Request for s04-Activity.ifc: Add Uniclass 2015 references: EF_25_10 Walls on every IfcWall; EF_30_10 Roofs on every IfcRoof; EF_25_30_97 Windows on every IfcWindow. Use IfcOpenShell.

First a look at what the model holds.

```python
import ifcopenshell

model = ifcopenshell.open("s04-Activity.ifc")
print(model.schema)
print("classifications:", [c.Name for c in model.by_type("IfcClassification")])
for ifc_class in ("IfcDoor", "IfcRoof", "IfcStair", "IfcWall", "IfcWindow"):
    print(ifc_class, len(model.by_type(ifc_class)))
```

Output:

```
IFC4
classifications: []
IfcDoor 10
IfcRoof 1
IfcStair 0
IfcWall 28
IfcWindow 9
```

```python
import ifcopenshell
import ifcopenshell.api.classification

model = ifcopenshell.open("s04-Activity.ifc")

system = ifcopenshell.api.classification.add_classification(model, classification="Uniclass 2015")

codes = {
    "IfcWall": ("EF_25_10", "Walls"),
    "IfcRoof": ("EF_30_10", "Roofs"),
    "IfcWindow": ("EF_25_30_97", "Windows"),
}
for ifc_class, (code, name) in codes.items():
    products = model.by_type(ifc_class)
    ifcopenshell.api.classification.add_reference(
        model, products=products, classification=system, identification=code, name=name
    )
    print(code, len(products))

model.write("s04-Activity_edited.ifc")
```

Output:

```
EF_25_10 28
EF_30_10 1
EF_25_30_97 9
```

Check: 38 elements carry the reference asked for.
